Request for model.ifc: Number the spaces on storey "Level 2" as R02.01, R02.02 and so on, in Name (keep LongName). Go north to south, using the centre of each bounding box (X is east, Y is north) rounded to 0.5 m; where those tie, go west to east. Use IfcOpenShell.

First a look at what the model holds.

```python
import ifcopenshell
import ifcopenshell.util.element
import ifcopenshell.util.placement

model = ifcopenshell.open("model.ifc")
print(model.schema)
storey = next(s for s in model.by_type("IfcBuildingStorey") if s.Name == "Level 2")
spaces = [e for e in ifcopenshell.util.element.get_decomposition(storey) if e.is_a("IfcSpace")]
for e in sorted(spaces, key=lambda e: e.id()):
    origin = ifcopenshell.util.placement.get_local_placement(e.ObjectPlacement)[:3, 3]
    print(e.id(), e.Name, e.LongName, origin.round(2) + 0.0, sep=" | ")
```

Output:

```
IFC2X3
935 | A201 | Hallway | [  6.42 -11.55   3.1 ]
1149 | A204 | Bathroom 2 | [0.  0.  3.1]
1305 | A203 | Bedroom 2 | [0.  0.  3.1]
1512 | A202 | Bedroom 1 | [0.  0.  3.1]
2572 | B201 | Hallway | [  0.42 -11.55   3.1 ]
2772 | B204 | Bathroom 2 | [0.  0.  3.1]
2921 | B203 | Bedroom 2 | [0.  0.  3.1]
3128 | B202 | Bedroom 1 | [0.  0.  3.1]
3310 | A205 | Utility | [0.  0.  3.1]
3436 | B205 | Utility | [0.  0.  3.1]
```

```python
import ifcopenshell
import ifcopenshell.geom
import ifcopenshell.util.element
import ifcopenshell.util.shape

model = ifcopenshell.open("model.ifc")
settings = ifcopenshell.geom.settings()
settings.set("use-world-coords", True)


def centre(element):
    shape = ifcopenshell.geom.create_shape(settings, element)
    return ifcopenshell.util.shape.get_bbox_centroid(shape.geometry)


storey = next(s for s in model.by_type("IfcBuildingStorey") if s.Name == "Level 2")
spaces = [e for e in ifcopenshell.util.element.get_decomposition(storey) if e.is_a("IfcSpace")]

# Insertion points can sit at a corner or the storey origin, so sort by the geometry (in metres).
centres = {e: centre(e) for e in spaces}
spaces.sort(key=lambda e: (-round(centres[e][1] / 0.5), centres[e][0]))

for i, e in enumerate(spaces, start=1):
    number = f"R02.{i:02d}"
    e.Name = number
    print(e.id(), number)

model.write("model_v2.ifc")
```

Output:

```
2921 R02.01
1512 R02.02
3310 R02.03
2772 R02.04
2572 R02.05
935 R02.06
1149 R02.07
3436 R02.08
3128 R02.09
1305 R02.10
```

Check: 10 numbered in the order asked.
